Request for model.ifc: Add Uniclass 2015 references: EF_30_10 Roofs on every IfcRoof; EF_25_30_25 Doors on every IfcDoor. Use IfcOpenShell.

First a look at what the model holds.

```python
import ifcopenshell

model = ifcopenshell.open("model.ifc")
print(model.schema)
print("classifications:", [c.Name for c in model.by_type("IfcClassification")])
for ifc_class in ("IfcDoor", "IfcRoof", "IfcStair", "IfcWall", "IfcWindow"):
    print(ifc_class, len(model.by_type(ifc_class)))
```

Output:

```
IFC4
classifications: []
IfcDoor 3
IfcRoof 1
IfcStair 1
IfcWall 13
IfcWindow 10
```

```python
import ifcopenshell
import ifcopenshell.api.classification

model = ifcopenshell.open("model.ifc")

system = ifcopenshell.api.classification.add_classification(model, classification="Uniclass 2015")

codes = {
    "IfcRoof": ("EF_30_10", "Roofs"),
    "IfcDoor": ("EF_25_30_25", "Doors"),
}
for ifc_class, (code, name) in codes.items():
    products = model.by_type(ifc_class)
    ifcopenshell.api.classification.add_reference(
        model, products=products, classification=system, identification=code, name=name
    )
    print(code, len(products))

model.write("model-out.ifc")
```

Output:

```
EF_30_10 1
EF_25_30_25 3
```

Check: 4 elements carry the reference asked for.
